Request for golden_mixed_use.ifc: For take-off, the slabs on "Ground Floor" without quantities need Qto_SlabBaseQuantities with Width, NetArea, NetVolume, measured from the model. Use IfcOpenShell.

First a look at what the model holds.

```python
import ifcopenshell
import ifcopenshell.util.element
import ifcopenshell.util.unit

model = ifcopenshell.open("golden_mixed_use.ifc")
print(model.schema)
for unit_type in ("LENGTHUNIT", "AREAUNIT", "VOLUMEUNIT"):
    print(unit_type, ifcopenshell.util.unit.calculate_unit_scale(model, unit_type))
storey = next(s for s in model.by_type("IfcBuildingStorey") if s.Name == "Ground Floor")
slabs = [e for e in ifcopenshell.util.element.get_decomposition(storey) if e.is_a("IfcSlab")]
for e in sorted(slabs, key=lambda e: e.id()):
    print(e.id(), e.is_a(), e.Name, list(ifcopenshell.util.element.get_psets(e, qtos_only=True)), sep=" | ")
```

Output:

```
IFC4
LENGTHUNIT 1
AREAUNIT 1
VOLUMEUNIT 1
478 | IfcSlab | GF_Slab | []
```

```python
import ifcopenshell
import ifcopenshell.api.pset
import ifcopenshell.geom
import ifcopenshell.util.element
import ifcopenshell.util.shape
import ifcopenshell.util.unit

model = ifcopenshell.open("golden_mixed_use.ifc")
unit_scale = ifcopenshell.util.unit.calculate_unit_scale(model)
area_scale = ifcopenshell.util.unit.calculate_unit_scale(model, "AREAUNIT")
volume_scale = ifcopenshell.util.unit.calculate_unit_scale(model, "VOLUMEUNIT")
settings = ifcopenshell.geom.settings()

storey = next(s for s in model.by_type("IfcBuildingStorey") if s.Name == "Ground Floor")
slabs = [e for e in ifcopenshell.util.element.get_decomposition(storey) if e.is_a("IfcSlab")]

for e in sorted(slabs, key=lambda e: e.id()):
    if ifcopenshell.util.element.get_psets(e, qtos_only=True, should_inherit=False):
        continue
    # Geometry comes back in metres, in the element's own axes.
    shape = ifcopenshell.geom.create_shape(settings, e)
    values = {
        "Width": ifcopenshell.util.shape.get_z(shape.geometry) / unit_scale,
        "NetArea": ifcopenshell.util.shape.get_footprint_area(shape.geometry) / area_scale,
        "NetVolume": ifcopenshell.util.shape.get_volume(shape.geometry) / volume_scale,
    }
    qto = ifcopenshell.api.pset.add_qto(model, product=e, name="Qto_SlabBaseQuantities")
    ifcopenshell.api.pset.edit_qto(model, qto=qto, properties=values)
    print(e.id(), {k: round(v, 3) for k, v in values.items()})

model.write("golden_mixed_use-out.ifc")
```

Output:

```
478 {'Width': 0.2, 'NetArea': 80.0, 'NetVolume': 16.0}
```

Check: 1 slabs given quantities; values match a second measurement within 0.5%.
